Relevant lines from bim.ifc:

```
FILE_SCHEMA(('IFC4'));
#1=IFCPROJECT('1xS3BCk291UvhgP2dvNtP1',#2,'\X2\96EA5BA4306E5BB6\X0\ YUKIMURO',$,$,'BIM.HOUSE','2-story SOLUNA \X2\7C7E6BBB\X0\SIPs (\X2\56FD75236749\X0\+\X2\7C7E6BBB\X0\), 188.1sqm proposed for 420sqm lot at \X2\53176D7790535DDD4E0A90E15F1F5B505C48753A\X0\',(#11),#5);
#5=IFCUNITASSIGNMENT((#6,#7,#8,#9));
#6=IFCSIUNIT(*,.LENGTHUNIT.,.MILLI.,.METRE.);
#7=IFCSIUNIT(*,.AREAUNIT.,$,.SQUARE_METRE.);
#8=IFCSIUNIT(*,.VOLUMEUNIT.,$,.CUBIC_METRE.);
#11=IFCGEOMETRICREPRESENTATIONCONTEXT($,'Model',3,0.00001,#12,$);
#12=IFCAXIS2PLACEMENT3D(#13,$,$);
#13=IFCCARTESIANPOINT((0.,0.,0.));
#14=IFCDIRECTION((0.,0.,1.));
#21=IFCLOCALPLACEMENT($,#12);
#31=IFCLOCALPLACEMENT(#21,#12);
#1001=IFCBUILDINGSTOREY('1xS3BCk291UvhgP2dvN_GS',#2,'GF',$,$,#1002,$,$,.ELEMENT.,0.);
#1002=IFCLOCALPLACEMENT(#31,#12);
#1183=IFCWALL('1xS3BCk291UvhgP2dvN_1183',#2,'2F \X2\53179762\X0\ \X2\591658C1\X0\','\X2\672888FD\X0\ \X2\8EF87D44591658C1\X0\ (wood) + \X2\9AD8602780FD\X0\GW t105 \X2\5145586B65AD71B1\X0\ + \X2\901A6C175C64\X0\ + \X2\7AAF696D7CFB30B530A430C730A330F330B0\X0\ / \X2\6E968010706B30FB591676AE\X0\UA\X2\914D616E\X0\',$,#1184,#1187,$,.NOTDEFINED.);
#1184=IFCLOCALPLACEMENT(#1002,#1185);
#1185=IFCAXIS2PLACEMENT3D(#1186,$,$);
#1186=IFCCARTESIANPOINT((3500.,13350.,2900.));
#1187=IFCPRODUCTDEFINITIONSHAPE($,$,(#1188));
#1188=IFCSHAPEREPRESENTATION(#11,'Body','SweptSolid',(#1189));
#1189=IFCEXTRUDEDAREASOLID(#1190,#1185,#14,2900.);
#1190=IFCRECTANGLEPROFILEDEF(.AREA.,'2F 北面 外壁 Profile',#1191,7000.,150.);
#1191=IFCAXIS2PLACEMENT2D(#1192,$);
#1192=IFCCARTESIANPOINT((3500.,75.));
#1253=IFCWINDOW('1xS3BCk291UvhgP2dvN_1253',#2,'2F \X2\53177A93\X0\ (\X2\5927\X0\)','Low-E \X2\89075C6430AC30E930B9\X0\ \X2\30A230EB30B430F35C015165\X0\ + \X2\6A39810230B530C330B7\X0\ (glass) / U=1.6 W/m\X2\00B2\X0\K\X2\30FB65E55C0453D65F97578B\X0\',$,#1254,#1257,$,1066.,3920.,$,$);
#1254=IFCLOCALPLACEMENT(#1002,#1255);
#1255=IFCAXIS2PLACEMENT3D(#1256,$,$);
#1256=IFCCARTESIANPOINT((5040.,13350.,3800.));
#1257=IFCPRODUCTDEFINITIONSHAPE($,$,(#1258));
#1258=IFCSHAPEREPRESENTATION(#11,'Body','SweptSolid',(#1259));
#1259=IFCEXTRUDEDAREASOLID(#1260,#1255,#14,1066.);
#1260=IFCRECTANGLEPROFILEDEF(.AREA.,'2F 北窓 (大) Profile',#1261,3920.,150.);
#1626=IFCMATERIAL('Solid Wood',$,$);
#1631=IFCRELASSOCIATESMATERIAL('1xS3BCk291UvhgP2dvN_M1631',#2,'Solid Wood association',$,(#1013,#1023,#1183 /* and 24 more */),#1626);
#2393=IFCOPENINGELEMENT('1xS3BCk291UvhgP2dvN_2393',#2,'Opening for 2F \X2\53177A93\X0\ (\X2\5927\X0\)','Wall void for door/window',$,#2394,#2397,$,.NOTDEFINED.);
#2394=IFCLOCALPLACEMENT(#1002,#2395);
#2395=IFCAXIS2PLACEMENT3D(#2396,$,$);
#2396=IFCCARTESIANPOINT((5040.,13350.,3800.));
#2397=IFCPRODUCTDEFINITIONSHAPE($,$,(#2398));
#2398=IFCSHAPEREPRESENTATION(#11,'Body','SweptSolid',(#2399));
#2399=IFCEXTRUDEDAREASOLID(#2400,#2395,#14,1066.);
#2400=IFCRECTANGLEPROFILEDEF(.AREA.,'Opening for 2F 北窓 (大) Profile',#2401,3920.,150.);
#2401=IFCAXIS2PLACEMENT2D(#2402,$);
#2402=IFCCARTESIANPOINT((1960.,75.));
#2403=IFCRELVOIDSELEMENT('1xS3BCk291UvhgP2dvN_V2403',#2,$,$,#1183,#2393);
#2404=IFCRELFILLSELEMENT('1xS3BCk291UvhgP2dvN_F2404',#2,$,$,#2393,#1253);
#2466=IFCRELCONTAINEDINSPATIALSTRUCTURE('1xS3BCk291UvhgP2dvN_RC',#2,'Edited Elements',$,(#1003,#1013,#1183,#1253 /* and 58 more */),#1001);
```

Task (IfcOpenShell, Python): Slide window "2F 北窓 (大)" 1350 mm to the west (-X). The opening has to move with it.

```python
import ifcopenshell
import ifcopenshell.api.geometry
import ifcopenshell.util.placement
import ifcopenshell.util.unit

model = ifcopenshell.open("bim.ifc")
unit_scale = ifcopenshell.util.unit.calculate_unit_scale(model)

window = model.by_guid("1xS3BCk291UvhgP2dvN_1253")
opening = window.FillsVoids[0].RelatingOpeningElement
wall = opening.VoidsElements[0].RelatingBuildingElement

wall_matrix = ifcopenshell.util.placement.get_local_placement(wall.ObjectPlacement)
shift = wall_matrix[:3, 0] * -1.35 / unit_scale
before = ifcopenshell.util.placement.get_local_placement(window.ObjectPlacement)[:3, 3].copy()

# The window is not placed relative to its opening, so move both.
for product in (opening, window):
    matrix = ifcopenshell.util.placement.get_local_placement(product.ObjectPlacement)
    matrix[:3, 3] += shift
    ifcopenshell.api.geometry.edit_object_placement(model, product=product, matrix=matrix, is_si=False)

after = ifcopenshell.util.placement.get_local_placement(window.ObjectPlacement)[:3, 3]
print("window moved by", (after - before).round(3) + 0.0)

model.write("bim_rev.ifc")
```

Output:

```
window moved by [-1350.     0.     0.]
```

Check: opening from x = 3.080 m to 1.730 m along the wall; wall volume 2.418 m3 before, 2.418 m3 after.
